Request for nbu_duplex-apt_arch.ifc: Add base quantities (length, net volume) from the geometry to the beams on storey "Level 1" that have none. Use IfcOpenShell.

First a look at what the model holds.

```python
import ifcopenshell
import ifcopenshell.util.element
import ifcopenshell.util.unit

model = ifcopenshell.open("nbu_duplex-apt_arch.ifc")
print(model.schema)
for unit_type in ("LENGTHUNIT", "AREAUNIT", "VOLUMEUNIT"):
    print(unit_type, ifcopenshell.util.unit.calculate_unit_scale(model, unit_type))
storey = next(s for s in model.by_type("IfcBuildingStorey") if s.Name == "Level 1")
beams = [e for e in ifcopenshell.util.element.get_decomposition(storey) if e.is_a("IfcBeam")]
for e in sorted(beams, key=lambda e: e.id()):
    print(e.id(), e.is_a(), e.Name, list(ifcopenshell.util.element.get_psets(e, qtos_only=True)), sep=" | ")
```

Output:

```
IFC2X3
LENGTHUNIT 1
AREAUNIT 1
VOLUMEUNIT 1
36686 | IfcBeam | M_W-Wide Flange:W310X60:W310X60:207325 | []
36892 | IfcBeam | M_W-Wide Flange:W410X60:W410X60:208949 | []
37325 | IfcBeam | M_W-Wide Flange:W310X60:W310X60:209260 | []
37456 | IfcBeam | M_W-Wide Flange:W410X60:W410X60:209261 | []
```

```python
import ifcopenshell
import ifcopenshell.api.pset
import ifcopenshell.geom
import ifcopenshell.util.element
import ifcopenshell.util.shape
import ifcopenshell.util.unit

model = ifcopenshell.open("nbu_duplex-apt_arch.ifc")
unit_scale = ifcopenshell.util.unit.calculate_unit_scale(model)
volume_scale = ifcopenshell.util.unit.calculate_unit_scale(model, "VOLUMEUNIT")
settings = ifcopenshell.geom.settings()

storey = next(s for s in model.by_type("IfcBuildingStorey") if s.Name == "Level 1")
beams = [e for e in ifcopenshell.util.element.get_decomposition(storey) if e.is_a("IfcBeam")]

for e in sorted(beams, key=lambda e: e.id()):
    if ifcopenshell.util.element.get_psets(e, qtos_only=True, should_inherit=False):
        continue
    # Geometry comes back in metres, in the element's own axes.
    shape = ifcopenshell.geom.create_shape(settings, e)
    values = {
        "Length": ifcopenshell.util.shape.get_max_xyz(shape.geometry) / unit_scale,
        "NetVolume": ifcopenshell.util.shape.get_volume(shape.geometry) / volume_scale,
    }
    qto = ifcopenshell.api.pset.add_qto(model, product=e, name="BaseQuantities")
    ifcopenshell.api.pset.edit_qto(model, qto=qto, properties=values)
    print(e.id(), {k: round(v, 3) for k, v in values.items()})

model.write("nbu_duplex-apt_arch_updated.ifc")
```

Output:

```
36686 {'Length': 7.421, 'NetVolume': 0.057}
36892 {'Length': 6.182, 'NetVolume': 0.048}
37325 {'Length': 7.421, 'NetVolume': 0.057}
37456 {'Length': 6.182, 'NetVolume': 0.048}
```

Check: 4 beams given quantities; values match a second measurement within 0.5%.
